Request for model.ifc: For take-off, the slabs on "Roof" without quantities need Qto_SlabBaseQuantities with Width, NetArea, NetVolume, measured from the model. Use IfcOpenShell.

First a look at what the model holds.

```python
import ifcopenshell
import ifcopenshell.util.element
import ifcopenshell.util.unit

model = ifcopenshell.open("model.ifc")
print(model.schema)
for unit_type in ("LENGTHUNIT", "AREAUNIT", "VOLUMEUNIT"):
    print(unit_type, ifcopenshell.util.unit.calculate_unit_scale(model, unit_type))
storey = next(s for s in model.by_type("IfcBuildingStorey") if s.Name == "Roof")
slabs = [e for e in ifcopenshell.util.element.get_decomposition(storey) if e.is_a("IfcSlab")]
for e in sorted(slabs, key=lambda e: e.id()):
    print(e.id(), e.is_a(), e.Name, list(ifcopenshell.util.element.get_psets(e, qtos_only=True)), sep=" | ")
```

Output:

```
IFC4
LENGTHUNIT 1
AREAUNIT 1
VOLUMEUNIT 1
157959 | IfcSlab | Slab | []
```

```python
import ifcopenshell
import ifcopenshell.api.pset
import ifcopenshell.geom
import ifcopenshell.util.element
import ifcopenshell.util.shape
import ifcopenshell.util.unit

model = ifcopenshell.open("model.ifc")
unit_scale = ifcopenshell.util.unit.calculate_unit_scale(model)
area_scale = ifcopenshell.util.unit.calculate_unit_scale(model, "AREAUNIT")
volume_scale = ifcopenshell.util.unit.calculate_unit_scale(model, "VOLUMEUNIT")
settings = ifcopenshell.geom.settings()

storey = next(s for s in model.by_type("IfcBuildingStorey") if s.Name == "Roof")
slabs = [e for e in ifcopenshell.util.element.get_decomposition(storey) if e.is_a("IfcSlab")]

for e in sorted(slabs, key=lambda e: e.id()):
    if ifcopenshell.util.element.get_psets(e, qtos_only=True, should_inherit=False):
        continue
    # Geometry comes back in metres, in the element's own axes.
    shape = ifcopenshell.geom.create_shape(settings, e)
    values = {
        "Width": ifcopenshell.util.shape.get_z(shape.geometry) / unit_scale,
        "NetArea": ifcopenshell.util.shape.get_footprint_area(shape.geometry) / area_scale,
        "NetVolume": ifcopenshell.util.shape.get_volume(shape.geometry) / volume_scale,
    }
    qto = ifcopenshell.api.pset.add_qto(model, product=e, name="Qto_SlabBaseQuantities")
    ifcopenshell.api.pset.edit_qto(model, qto=qto, properties=values)
    print(e.id(), {k: round(v, 3) for k, v in values.items()})

model.write("model-out.ifc")
```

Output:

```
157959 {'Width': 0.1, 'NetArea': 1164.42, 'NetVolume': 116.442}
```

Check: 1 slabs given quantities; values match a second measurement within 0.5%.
